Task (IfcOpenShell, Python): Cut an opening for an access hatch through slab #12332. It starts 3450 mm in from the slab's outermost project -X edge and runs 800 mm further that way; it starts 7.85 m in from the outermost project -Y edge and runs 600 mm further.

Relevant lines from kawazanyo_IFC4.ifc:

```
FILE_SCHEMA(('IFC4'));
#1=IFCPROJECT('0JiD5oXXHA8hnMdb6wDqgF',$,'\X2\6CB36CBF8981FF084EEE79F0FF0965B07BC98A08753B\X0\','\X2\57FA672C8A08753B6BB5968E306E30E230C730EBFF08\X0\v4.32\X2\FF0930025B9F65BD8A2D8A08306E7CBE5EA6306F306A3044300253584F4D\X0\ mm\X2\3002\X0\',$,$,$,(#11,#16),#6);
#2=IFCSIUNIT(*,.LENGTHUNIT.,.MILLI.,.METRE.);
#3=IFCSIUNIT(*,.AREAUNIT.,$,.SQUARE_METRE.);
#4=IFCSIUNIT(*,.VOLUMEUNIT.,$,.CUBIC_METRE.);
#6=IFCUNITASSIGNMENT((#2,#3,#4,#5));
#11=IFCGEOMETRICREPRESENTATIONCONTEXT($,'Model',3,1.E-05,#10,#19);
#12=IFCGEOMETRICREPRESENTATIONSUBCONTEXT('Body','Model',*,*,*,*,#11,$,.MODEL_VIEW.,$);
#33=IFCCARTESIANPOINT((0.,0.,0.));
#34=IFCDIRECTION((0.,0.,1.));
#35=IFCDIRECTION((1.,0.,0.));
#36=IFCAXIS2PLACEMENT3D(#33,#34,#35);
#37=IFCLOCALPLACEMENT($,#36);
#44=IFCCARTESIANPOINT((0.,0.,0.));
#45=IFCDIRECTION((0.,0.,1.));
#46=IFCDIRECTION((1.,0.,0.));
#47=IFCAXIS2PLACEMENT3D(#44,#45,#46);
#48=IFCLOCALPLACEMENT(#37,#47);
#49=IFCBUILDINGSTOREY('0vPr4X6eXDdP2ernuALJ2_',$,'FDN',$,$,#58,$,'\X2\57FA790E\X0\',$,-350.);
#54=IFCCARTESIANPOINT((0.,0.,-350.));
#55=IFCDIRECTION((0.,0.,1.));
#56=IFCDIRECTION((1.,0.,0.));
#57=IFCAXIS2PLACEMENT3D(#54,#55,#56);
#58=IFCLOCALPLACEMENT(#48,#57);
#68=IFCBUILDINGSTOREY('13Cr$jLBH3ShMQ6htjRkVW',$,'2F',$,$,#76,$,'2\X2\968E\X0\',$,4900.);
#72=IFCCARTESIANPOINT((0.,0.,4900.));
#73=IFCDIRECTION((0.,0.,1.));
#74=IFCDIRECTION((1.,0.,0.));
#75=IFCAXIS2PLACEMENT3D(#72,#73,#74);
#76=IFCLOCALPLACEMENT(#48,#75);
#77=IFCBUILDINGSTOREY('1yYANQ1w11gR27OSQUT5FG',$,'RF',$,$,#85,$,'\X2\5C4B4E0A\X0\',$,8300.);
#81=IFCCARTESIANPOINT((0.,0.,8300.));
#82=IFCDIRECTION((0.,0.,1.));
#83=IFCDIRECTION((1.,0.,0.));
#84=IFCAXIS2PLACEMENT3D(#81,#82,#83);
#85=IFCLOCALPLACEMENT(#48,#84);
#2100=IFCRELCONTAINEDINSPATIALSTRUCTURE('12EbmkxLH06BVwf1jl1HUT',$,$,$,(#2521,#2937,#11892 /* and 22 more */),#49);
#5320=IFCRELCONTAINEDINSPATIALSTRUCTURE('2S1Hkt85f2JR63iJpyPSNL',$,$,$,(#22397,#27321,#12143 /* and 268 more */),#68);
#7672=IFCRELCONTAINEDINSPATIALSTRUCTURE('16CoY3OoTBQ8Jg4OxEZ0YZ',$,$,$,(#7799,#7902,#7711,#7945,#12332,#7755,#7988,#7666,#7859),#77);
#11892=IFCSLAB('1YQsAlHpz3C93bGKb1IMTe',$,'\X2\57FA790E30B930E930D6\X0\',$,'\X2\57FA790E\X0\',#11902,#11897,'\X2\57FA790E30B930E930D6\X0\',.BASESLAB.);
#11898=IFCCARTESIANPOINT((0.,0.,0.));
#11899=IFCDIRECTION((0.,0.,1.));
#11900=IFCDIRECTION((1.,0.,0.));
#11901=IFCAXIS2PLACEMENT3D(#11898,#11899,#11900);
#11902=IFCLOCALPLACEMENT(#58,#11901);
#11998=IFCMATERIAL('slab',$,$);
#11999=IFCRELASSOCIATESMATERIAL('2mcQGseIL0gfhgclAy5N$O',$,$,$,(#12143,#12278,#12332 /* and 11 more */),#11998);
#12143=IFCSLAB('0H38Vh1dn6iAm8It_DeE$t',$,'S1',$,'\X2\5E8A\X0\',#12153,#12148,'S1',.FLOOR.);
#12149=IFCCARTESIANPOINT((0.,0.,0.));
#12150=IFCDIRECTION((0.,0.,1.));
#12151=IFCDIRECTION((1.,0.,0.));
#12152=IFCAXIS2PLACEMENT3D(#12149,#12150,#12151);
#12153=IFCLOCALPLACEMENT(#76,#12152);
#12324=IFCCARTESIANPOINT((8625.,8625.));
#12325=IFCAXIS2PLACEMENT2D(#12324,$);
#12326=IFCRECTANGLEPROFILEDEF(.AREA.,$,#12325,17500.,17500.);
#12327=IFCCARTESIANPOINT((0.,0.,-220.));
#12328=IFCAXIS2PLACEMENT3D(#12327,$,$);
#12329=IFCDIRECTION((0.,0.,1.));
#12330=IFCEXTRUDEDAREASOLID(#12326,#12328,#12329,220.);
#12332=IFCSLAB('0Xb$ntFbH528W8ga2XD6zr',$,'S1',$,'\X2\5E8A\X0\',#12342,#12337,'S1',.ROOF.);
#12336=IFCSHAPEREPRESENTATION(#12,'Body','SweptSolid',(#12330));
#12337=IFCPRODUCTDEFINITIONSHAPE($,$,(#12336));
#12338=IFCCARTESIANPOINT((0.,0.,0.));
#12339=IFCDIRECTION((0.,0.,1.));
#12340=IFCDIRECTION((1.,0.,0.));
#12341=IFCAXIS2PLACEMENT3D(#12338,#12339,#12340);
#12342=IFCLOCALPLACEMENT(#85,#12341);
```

```python
import numpy as np
import ifcopenshell
import ifcopenshell.api.feature
import ifcopenshell.api.geometry
import ifcopenshell.api.root
import ifcopenshell.geom
import ifcopenshell.util.placement
import ifcopenshell.util.representation
import ifcopenshell.util.shape
import ifcopenshell.util.unit

model = ifcopenshell.open("kawazanyo_IFC4.ifc")
unit_scale = ifcopenshell.util.unit.calculate_unit_scale(model)
settings = ifcopenshell.geom.settings()


def volume(element):
    """Net volume in cubic metres, openings subtracted."""
    shape = ifcopenshell.geom.create_shape(settings, element)
    return ifcopenshell.util.shape.get_volume(shape.geometry)


slab = model.by_guid("0Xb$ntFbH528W8ga2XD6zr")
before = volume(slab)

# Extent in the slab's own axes, in metres. The edges named are its -X and -Y sides.
slab_shape = ifcopenshell.geom.create_shape(settings, slab)
vertices = ifcopenshell.util.shape.get_vertices(slab_shape.geometry)
x_min, y_min, bottom = vertices.min(axis=0)
top = vertices[:, 2].max()

opening = ifcopenshell.api.root.create_entity(model, ifc_class="IfcOpeningElement", name="Access hatch opening", predefined_type="OPENING")
context = ifcopenshell.util.representation.get_context(model, "Model", "Body", "MODEL_VIEW")
width, depth = 0.8, 0.6
outline = [(0.0, 0.0), (width, 0.0), (width, depth), (0.0, depth), (0.0, 0.0)]
# Overshoot both faces by 50 mm so the cut is clean.
shape = ifcopenshell.api.geometry.add_slab_representation(
    model, context=context, depth=top - bottom + 0.1, polyline=outline
)
ifcopenshell.api.geometry.assign_representation(model, product=opening, representation=shape)

matrix = ifcopenshell.util.placement.get_local_placement(slab.ObjectPlacement)
matrix[:, 3] = matrix @ np.append(np.array([x_min + 3.45, y_min + 7.85, bottom - 0.05]) / unit_scale, 1.0)
ifcopenshell.api.geometry.edit_object_placement(model, product=opening, matrix=matrix, is_si=False)
ifcopenshell.api.feature.add_feature(model, feature=opening, element=slab)

after = volume(slab)

print(f"slab volume {before:.3f} -> {after:.3f} m3")

model.write("kawazanyo_IFC4_v2.ifc")
```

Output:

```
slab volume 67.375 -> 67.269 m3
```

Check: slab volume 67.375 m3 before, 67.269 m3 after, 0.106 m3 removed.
